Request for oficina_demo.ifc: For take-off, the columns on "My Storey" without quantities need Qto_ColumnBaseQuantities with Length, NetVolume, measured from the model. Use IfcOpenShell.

First a look at what the model holds.

```python
import ifcopenshell
import ifcopenshell.util.element
import ifcopenshell.util.unit

model = ifcopenshell.open("oficina_demo.ifc")
print(model.schema)
for unit_type in ("LENGTHUNIT", "AREAUNIT", "VOLUMEUNIT"):
    print(unit_type, ifcopenshell.util.unit.calculate_unit_scale(model, unit_type))
storey = next(s for s in model.by_type("IfcBuildingStorey") if s.Name == "My Storey")
columns = [e for e in ifcopenshell.util.element.get_decomposition(storey) if e.is_a("IfcColumn")]
for e in sorted(columns, key=lambda e: e.id()):
    print(e.id(), e.is_a(), e.Name, list(ifcopenshell.util.element.get_psets(e, qtos_only=True)), sep=" | ")
```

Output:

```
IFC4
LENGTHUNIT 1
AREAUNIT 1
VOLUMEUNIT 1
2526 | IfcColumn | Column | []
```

```python
import ifcopenshell
import ifcopenshell.api.pset
import ifcopenshell.geom
import ifcopenshell.util.element
import ifcopenshell.util.shape
import ifcopenshell.util.unit

model = ifcopenshell.open("oficina_demo.ifc")
unit_scale = ifcopenshell.util.unit.calculate_unit_scale(model)
volume_scale = ifcopenshell.util.unit.calculate_unit_scale(model, "VOLUMEUNIT")
settings = ifcopenshell.geom.settings()

storey = next(s for s in model.by_type("IfcBuildingStorey") if s.Name == "My Storey")
columns = [e for e in ifcopenshell.util.element.get_decomposition(storey) if e.is_a("IfcColumn")]

for e in sorted(columns, key=lambda e: e.id()):
    if ifcopenshell.util.element.get_psets(e, qtos_only=True, should_inherit=False):
        continue
    # Geometry comes back in metres, in the element's own axes.
    shape = ifcopenshell.geom.create_shape(settings, e)
    values = {
        "Length": ifcopenshell.util.shape.get_z(shape.geometry) / unit_scale,
        "NetVolume": ifcopenshell.util.shape.get_volume(shape.geometry) / volume_scale,
    }
    qto = ifcopenshell.api.pset.add_qto(model, product=e, name="Qto_ColumnBaseQuantities")
    ifcopenshell.api.pset.edit_qto(model, qto=qto, properties=values)
    print(e.id(), {k: round(v, 3) for k, v in values.items()})

model.write("oficina_demo_v2.ifc")
```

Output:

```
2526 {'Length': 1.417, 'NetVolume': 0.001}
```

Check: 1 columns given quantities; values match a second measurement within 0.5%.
